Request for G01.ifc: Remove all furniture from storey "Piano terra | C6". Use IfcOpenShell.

First a look at what the model holds.

```python
import ifcopenshell
import ifcopenshell.util.element

model = ifcopenshell.open("G01.ifc")
print(model.schema)
storey = next(s for s in model.by_type("IfcBuildingStorey") if s.Name == "Piano terra | C6")
furniture = [e for e in ifcopenshell.util.element.get_decomposition(storey) if e.is_a("IfcFurnishingElement")]
seen = {}
for e in furniture:
    element_type = ifcopenshell.util.element.get_type(e)
    name = element_type.Name if element_type not in (None, e) else None
    seen[name] = seen.get(name, 0) + 1
for name, count in sorted(seen.items(), key=str):
    print(count, "x", name)
```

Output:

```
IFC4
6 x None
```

```python
import ifcopenshell
import ifcopenshell.api.root
import ifcopenshell.util.element

model = ifcopenshell.open("G01.ifc")

storey = next(s for s in model.by_type("IfcBuildingStorey") if s.Name == "Piano terra | C6")
furniture = [e for e in ifcopenshell.util.element.get_decomposition(storey) if e.is_a("IfcFurnishingElement")]

for e in furniture:
    ifcopenshell.api.root.remove_product(model, product=e)
print(len(furniture), "removed")

model.write("G01_rev.ifc")
```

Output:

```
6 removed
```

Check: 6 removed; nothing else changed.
